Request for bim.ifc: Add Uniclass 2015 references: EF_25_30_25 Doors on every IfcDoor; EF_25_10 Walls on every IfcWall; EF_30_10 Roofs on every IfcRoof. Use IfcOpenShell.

First a look at what the model holds.

```python
import ifcopenshell

model = ifcopenshell.open("bim.ifc")
print(model.schema)
print("classifications:", [c.Name for c in model.by_type("IfcClassification")])
for ifc_class in ("IfcDoor", "IfcRoof", "IfcStair", "IfcWall", "IfcWindow"):
    print(ifc_class, len(model.by_type(ifc_class)))
```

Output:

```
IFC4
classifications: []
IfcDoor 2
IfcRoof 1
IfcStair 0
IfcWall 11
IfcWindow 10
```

```python
import ifcopenshell
import ifcopenshell.api.classification

model = ifcopenshell.open("bim.ifc")

system = ifcopenshell.api.classification.add_classification(model, classification="Uniclass 2015")

codes = {
    "IfcDoor": ("EF_25_30_25", "Doors"),
    "IfcWall": ("EF_25_10", "Walls"),
    "IfcRoof": ("EF_30_10", "Roofs"),
}
for ifc_class, (code, name) in codes.items():
    products = model.by_type(ifc_class)
    ifcopenshell.api.classification.add_reference(
        model, products=products, classification=system, identification=code, name=name
    )
    print(code, len(products))

model.write("bim_edited.ifc")
```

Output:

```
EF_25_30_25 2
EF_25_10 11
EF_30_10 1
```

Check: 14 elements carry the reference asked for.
